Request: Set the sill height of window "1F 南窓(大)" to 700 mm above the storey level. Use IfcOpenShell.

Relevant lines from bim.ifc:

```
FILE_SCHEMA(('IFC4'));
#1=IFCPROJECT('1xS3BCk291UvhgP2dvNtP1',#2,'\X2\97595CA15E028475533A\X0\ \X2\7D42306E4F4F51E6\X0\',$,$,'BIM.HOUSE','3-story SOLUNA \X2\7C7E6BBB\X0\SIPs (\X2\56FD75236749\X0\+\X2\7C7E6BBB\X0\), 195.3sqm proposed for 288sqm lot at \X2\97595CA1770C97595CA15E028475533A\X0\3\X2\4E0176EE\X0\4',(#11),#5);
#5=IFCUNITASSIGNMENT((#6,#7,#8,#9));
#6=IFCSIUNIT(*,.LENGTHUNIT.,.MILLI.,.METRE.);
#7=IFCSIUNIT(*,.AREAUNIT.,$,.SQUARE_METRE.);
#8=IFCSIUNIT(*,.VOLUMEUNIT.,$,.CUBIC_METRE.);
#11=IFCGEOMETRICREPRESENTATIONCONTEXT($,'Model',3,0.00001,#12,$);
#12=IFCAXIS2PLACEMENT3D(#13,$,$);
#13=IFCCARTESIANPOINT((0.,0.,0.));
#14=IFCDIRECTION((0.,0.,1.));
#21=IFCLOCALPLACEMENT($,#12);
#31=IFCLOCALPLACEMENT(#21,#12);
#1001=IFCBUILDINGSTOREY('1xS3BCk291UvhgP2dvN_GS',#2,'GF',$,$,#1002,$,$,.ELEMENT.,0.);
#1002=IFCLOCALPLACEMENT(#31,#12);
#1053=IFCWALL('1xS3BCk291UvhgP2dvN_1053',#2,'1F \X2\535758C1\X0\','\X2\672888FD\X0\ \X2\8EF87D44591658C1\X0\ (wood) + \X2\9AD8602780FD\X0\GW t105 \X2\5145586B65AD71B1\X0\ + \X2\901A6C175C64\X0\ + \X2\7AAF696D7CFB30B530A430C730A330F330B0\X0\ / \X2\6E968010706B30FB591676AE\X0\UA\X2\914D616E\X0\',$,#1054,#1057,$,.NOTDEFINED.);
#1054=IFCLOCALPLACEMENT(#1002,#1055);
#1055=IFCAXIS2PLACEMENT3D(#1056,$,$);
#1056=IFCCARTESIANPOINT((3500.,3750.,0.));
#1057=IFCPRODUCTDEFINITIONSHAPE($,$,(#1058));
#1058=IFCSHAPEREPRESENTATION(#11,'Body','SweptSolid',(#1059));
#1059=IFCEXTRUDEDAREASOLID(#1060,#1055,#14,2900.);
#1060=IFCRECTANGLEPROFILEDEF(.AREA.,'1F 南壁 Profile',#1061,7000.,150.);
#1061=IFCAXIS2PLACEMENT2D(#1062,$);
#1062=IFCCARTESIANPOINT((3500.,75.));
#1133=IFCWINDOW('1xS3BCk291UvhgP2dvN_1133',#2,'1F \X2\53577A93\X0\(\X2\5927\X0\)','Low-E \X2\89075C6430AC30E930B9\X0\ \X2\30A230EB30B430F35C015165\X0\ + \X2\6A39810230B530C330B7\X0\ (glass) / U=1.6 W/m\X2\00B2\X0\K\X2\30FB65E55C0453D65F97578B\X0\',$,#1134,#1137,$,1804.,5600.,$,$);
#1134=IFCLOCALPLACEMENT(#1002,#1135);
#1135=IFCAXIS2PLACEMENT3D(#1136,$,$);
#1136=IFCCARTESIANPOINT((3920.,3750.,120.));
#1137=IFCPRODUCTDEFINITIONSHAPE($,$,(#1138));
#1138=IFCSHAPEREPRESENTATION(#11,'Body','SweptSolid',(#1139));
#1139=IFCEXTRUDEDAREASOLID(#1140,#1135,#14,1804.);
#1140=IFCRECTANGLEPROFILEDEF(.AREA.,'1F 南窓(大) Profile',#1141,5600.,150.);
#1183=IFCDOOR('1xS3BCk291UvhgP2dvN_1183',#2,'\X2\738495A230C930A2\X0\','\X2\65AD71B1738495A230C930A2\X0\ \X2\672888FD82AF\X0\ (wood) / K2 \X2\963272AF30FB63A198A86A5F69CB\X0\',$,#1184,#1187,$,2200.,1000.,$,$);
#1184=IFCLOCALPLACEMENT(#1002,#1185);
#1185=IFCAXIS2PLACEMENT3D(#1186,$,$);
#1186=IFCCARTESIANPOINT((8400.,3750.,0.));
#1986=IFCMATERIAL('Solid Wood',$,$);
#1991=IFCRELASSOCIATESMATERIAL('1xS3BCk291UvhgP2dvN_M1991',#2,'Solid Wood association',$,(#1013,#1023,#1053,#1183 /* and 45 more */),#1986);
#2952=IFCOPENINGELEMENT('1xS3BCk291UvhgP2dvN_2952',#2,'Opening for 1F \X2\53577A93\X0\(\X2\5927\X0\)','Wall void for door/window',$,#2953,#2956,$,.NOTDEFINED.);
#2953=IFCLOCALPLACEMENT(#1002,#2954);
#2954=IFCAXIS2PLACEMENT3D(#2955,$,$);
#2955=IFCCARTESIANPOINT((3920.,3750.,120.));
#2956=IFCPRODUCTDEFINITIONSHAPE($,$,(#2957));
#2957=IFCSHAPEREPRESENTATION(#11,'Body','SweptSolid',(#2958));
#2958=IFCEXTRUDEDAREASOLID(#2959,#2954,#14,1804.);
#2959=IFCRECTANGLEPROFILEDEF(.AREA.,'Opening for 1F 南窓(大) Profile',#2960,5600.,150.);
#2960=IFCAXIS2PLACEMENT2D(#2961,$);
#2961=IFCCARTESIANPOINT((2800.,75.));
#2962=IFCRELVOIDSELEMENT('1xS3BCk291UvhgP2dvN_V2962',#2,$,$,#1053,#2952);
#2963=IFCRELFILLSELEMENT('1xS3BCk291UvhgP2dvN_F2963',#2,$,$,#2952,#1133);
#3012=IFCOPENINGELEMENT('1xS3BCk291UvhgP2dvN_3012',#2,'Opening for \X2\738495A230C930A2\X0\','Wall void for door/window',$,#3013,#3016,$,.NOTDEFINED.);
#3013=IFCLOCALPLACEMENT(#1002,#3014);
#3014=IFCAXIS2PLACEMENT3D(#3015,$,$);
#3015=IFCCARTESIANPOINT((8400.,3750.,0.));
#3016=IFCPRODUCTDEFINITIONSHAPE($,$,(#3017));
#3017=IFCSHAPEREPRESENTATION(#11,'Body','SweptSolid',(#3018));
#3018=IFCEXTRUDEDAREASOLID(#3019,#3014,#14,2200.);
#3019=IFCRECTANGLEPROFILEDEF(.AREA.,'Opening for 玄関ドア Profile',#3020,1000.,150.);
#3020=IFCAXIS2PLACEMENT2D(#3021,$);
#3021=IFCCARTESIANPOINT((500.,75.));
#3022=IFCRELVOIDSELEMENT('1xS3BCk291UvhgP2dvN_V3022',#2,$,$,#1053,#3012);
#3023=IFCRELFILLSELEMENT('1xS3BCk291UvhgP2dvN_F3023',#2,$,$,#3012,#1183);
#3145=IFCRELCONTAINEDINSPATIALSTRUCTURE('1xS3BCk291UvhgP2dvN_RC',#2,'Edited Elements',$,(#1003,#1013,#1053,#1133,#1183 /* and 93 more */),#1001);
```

```python
import numpy as np
import ifcopenshell
import ifcopenshell.api.geometry
import ifcopenshell.geom
import ifcopenshell.util.element
import ifcopenshell.util.placement
import ifcopenshell.util.shape
import ifcopenshell.util.unit

model = ifcopenshell.open("bim.ifc")
unit_scale = ifcopenshell.util.unit.calculate_unit_scale(model)

window = model.by_id(1133)
opening = window.FillsVoids[0].RelatingOpeningElement
storey = ifcopenshell.util.element.get_container(window, ifc_class="IfcBuildingStorey")
level = ifcopenshell.util.placement.get_local_placement(storey.ObjectPlacement)[2, 3]

# The opening's origin need not be at the sill, so measure its lowest point.
shape = ifcopenshell.geom.create_shape(ifcopenshell.geom.settings(), opening)
bottom = ifcopenshell.util.shape.get_shape_bottom_elevation(shape, shape.geometry) / unit_scale
dz = level + 700.0 - bottom

shift = np.array([0.0, 0.0, dz])
# The window is not placed relative to its opening, so move both.
for product in (opening, window):
    matrix = ifcopenshell.util.placement.get_local_placement(product.ObjectPlacement)
    matrix[:3, 3] += shift
    ifcopenshell.api.geometry.edit_object_placement(model, product=product, matrix=matrix, is_si=False)

print(f"moved by {dz * unit_scale:+.3f} m")

model.write("bim_v2.ifc")
```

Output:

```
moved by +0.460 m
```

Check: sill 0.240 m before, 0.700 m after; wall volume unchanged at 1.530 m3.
